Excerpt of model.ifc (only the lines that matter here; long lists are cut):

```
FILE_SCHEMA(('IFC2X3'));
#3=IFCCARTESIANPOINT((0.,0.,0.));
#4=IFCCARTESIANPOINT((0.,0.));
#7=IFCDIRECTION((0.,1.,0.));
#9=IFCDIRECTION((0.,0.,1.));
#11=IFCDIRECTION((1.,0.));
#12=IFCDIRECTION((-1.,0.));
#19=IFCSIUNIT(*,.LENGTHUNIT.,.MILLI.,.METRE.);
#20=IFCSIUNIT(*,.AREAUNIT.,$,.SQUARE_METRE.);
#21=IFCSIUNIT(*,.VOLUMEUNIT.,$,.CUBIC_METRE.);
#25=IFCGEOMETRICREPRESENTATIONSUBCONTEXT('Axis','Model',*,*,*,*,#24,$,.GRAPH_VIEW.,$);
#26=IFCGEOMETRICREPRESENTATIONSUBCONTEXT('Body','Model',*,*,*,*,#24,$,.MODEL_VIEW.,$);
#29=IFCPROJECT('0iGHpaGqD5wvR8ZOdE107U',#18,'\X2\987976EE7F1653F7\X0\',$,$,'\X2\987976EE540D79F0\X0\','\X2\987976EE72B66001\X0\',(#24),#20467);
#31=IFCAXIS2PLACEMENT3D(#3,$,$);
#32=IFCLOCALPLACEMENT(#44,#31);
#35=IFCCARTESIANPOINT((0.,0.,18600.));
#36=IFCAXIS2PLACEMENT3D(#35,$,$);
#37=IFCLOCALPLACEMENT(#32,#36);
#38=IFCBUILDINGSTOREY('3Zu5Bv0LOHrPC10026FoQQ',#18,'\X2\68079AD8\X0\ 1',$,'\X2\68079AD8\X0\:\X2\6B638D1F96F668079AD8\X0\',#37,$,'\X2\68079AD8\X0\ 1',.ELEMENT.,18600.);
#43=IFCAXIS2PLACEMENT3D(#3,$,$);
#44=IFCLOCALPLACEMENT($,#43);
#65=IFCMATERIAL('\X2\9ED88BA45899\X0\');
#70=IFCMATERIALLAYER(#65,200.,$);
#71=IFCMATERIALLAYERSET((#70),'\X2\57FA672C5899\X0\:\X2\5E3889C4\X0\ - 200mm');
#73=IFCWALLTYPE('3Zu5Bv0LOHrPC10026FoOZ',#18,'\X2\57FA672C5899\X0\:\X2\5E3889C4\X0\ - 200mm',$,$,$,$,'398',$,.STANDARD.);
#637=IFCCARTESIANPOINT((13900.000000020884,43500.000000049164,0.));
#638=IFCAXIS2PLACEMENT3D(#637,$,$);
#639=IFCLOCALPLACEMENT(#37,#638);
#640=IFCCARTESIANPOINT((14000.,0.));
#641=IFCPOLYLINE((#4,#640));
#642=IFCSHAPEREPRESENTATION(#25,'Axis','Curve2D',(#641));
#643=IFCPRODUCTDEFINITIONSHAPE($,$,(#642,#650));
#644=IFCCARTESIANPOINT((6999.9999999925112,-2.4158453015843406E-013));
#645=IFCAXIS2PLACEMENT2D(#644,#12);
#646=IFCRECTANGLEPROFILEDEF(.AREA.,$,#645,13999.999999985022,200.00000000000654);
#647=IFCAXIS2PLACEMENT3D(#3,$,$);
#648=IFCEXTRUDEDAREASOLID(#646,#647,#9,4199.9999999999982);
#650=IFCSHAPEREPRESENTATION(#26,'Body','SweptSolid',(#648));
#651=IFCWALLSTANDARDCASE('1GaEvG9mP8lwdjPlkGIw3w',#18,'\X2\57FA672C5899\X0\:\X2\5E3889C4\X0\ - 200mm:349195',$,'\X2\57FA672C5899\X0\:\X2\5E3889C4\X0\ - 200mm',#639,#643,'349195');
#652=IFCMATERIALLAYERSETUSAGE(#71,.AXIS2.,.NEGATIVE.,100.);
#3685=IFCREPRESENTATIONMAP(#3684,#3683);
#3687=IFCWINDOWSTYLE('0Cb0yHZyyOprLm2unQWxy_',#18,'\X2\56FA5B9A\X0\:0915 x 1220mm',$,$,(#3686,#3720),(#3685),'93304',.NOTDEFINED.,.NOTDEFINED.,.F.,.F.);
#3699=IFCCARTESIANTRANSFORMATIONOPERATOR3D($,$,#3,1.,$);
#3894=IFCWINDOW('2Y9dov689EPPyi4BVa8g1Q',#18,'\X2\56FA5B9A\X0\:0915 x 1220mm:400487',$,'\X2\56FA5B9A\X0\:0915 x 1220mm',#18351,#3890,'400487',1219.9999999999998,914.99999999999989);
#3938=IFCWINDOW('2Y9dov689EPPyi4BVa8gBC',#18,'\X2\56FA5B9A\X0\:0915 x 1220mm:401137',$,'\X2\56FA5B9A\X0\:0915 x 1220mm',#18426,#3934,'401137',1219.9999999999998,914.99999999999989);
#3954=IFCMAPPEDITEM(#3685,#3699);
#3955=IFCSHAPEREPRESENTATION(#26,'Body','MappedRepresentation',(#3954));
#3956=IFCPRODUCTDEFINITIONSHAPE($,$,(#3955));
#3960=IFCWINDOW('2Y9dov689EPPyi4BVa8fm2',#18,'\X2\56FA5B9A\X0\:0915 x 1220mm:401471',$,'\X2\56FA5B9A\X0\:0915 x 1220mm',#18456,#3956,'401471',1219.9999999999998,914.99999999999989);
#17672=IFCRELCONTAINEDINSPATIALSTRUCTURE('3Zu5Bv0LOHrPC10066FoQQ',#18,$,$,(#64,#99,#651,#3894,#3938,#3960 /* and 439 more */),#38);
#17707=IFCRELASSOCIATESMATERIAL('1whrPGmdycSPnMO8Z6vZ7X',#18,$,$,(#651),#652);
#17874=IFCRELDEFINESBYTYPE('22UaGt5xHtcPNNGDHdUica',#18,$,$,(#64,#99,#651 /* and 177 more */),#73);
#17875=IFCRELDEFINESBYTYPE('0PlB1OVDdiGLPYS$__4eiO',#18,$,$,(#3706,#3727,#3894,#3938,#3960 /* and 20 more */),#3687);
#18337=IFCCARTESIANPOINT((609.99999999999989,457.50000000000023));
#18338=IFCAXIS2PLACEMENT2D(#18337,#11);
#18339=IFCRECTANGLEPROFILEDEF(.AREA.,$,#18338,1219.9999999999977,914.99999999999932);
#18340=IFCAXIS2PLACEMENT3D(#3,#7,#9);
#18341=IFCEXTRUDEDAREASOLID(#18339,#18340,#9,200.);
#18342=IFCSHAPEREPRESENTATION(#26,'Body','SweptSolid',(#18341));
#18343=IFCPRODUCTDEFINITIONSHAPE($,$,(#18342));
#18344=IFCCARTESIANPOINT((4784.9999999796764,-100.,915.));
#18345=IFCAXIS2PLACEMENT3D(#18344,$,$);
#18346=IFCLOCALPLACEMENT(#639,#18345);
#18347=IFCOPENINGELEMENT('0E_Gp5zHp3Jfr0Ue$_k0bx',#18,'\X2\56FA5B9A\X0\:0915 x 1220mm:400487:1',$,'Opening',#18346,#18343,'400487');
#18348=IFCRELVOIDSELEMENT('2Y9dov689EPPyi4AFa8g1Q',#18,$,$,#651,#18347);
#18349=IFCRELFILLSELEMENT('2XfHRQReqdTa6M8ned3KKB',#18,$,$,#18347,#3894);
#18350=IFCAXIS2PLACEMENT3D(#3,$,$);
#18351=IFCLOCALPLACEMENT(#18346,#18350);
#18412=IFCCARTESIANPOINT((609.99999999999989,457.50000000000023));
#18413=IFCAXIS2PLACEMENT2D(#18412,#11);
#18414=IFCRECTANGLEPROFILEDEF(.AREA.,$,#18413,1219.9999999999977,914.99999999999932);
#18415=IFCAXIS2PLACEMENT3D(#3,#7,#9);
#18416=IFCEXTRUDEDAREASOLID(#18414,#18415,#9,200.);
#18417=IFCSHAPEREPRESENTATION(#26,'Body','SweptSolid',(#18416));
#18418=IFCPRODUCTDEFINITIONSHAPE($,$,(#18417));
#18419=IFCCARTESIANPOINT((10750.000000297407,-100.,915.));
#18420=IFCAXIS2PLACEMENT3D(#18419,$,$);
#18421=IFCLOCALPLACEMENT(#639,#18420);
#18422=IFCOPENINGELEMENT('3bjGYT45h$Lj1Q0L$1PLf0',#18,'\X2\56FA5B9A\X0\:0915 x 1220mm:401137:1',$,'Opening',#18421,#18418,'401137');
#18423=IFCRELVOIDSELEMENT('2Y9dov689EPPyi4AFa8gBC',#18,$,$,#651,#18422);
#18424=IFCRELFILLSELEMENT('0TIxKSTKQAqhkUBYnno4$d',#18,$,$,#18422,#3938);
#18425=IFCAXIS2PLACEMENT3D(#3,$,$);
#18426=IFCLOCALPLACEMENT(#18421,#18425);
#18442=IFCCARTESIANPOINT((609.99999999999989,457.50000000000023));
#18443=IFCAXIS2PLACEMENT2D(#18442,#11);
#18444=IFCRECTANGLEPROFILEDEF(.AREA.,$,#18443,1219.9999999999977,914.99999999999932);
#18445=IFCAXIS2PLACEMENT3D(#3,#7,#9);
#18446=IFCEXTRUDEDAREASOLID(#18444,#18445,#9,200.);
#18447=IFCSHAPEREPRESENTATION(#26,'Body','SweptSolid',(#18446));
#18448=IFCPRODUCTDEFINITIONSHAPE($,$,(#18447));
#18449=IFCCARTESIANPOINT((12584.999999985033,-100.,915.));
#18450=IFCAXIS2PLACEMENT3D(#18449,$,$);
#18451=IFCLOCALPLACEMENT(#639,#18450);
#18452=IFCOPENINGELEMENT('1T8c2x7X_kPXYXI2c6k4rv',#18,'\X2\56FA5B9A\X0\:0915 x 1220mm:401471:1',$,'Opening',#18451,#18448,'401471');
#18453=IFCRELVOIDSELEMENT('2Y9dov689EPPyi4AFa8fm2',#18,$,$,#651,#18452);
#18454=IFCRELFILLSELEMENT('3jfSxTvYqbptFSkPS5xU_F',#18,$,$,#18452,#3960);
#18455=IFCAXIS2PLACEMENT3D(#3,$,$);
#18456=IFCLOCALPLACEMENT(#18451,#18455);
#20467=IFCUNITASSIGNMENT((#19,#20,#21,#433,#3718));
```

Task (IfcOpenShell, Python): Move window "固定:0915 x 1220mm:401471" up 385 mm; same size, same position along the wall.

```python
import numpy as np
import ifcopenshell
import ifcopenshell.api.geometry
import ifcopenshell.util.placement
import ifcopenshell.util.unit

model = ifcopenshell.open("model.ifc")
unit_scale = ifcopenshell.util.unit.calculate_unit_scale(model)

window = model.by_guid("2Y9dov689EPPyi4BVa8fm2")
opening = window.FillsVoids[0].RelatingOpeningElement
dz = 0.385 / unit_scale

shift = np.array([0.0, 0.0, dz])
# The window is placed relative to its opening, so it follows when the opening moves.
matrix = ifcopenshell.util.placement.get_local_placement(opening.ObjectPlacement)
matrix[:3, 3] += shift
ifcopenshell.api.geometry.edit_object_placement(
    model, product=opening, matrix=matrix, is_si=False, should_transform_children=True
)

print(f"moved by {dz * unit_scale:+.3f} m")

model.write("model-out.ifc")
```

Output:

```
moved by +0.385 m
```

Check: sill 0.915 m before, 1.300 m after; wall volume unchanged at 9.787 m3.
